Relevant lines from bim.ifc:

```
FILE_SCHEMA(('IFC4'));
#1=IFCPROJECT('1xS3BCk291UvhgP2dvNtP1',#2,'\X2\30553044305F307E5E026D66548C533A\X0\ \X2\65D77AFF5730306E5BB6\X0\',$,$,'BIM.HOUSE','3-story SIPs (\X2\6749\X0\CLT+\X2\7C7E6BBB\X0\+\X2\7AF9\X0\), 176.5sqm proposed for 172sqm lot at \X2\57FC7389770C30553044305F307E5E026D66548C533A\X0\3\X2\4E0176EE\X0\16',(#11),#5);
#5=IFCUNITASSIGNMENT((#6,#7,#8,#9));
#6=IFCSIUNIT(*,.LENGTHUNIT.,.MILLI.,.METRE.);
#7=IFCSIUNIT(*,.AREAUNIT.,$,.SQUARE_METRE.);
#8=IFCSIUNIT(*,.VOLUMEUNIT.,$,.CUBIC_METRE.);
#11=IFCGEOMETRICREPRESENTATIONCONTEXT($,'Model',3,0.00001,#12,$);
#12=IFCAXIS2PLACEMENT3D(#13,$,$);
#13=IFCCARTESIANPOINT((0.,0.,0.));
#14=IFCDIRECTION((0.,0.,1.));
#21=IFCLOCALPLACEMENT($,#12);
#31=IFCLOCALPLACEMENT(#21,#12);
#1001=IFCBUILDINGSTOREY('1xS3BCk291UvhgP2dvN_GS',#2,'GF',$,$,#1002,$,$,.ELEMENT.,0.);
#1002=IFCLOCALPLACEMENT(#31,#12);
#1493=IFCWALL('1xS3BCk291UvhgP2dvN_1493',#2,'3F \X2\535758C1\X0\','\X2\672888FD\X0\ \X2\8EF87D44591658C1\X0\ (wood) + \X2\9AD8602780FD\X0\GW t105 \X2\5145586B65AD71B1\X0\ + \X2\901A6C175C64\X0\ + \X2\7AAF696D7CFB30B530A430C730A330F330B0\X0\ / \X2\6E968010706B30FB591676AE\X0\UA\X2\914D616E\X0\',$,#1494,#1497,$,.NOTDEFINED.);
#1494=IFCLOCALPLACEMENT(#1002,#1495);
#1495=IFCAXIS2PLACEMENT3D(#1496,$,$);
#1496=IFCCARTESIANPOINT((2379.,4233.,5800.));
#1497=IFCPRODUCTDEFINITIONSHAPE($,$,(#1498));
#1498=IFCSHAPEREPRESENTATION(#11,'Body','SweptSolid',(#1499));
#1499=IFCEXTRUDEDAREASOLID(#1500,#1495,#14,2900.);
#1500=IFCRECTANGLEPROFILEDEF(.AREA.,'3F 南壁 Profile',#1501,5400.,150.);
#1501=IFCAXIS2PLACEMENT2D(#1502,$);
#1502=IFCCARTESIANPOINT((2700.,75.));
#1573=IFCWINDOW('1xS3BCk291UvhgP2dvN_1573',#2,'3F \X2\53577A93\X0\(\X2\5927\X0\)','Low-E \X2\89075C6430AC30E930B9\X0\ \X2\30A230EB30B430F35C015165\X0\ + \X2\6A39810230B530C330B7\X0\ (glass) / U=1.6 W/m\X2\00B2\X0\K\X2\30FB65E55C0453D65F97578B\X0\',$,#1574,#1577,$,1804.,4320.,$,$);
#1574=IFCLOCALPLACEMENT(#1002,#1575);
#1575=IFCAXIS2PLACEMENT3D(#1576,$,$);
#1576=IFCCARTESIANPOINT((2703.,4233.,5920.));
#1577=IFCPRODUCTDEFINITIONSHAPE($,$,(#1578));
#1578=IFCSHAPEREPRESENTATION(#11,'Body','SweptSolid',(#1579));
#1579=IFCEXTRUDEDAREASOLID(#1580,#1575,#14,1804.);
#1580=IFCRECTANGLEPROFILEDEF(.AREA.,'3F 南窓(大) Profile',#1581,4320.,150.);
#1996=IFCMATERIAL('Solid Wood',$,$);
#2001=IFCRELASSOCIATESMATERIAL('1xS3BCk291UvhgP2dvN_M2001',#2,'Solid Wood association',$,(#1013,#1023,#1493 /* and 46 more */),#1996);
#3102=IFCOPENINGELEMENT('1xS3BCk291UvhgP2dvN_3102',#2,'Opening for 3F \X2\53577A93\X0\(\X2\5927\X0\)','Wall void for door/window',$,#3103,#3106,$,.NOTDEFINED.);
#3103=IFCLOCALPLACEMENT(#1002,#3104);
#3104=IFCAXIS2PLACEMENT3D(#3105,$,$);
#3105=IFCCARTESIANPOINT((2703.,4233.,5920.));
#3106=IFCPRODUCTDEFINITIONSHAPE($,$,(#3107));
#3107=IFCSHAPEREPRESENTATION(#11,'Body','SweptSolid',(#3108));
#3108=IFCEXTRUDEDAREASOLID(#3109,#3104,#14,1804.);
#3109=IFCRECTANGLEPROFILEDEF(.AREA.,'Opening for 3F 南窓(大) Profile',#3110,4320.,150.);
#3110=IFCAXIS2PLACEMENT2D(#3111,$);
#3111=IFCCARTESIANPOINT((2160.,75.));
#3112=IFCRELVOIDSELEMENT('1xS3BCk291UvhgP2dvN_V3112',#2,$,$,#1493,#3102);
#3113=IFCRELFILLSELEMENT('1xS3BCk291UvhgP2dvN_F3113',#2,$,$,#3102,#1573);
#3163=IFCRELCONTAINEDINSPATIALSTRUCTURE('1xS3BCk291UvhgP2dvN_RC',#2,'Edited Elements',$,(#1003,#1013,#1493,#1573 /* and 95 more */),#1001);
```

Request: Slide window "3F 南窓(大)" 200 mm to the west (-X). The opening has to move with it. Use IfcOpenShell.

```python
import ifcopenshell
import ifcopenshell.api.geometry
import ifcopenshell.util.placement

model = ifcopenshell.open("bim.ifc")

window = model.by_guid("1xS3BCk291UvhgP2dvN_1573")
opening = window.FillsVoids[0].RelatingOpeningElement
wall = opening.VoidsElements[0].RelatingBuildingElement

wall_matrix = ifcopenshell.util.placement.get_local_placement(wall.ObjectPlacement)
shift = wall_matrix[:3, 0] * -200.0
before = ifcopenshell.util.placement.get_local_placement(window.ObjectPlacement)[:3, 3].copy()

# The window is not placed relative to its opening, so move both.
for product in (opening, window):
    matrix = ifcopenshell.util.placement.get_local_placement(product.ObjectPlacement)
    matrix[:3, 3] += shift
    ifcopenshell.api.geometry.edit_object_placement(model, product=product, matrix=matrix, is_si=False)

after = ifcopenshell.util.placement.get_local_placement(window.ObjectPlacement)[:3, 3]
print("window moved by", (after - before).round(3) + 0.0)

model.write("bim-out.ifc")
```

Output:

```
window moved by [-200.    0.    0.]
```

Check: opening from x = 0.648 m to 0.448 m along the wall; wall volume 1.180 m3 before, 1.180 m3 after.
